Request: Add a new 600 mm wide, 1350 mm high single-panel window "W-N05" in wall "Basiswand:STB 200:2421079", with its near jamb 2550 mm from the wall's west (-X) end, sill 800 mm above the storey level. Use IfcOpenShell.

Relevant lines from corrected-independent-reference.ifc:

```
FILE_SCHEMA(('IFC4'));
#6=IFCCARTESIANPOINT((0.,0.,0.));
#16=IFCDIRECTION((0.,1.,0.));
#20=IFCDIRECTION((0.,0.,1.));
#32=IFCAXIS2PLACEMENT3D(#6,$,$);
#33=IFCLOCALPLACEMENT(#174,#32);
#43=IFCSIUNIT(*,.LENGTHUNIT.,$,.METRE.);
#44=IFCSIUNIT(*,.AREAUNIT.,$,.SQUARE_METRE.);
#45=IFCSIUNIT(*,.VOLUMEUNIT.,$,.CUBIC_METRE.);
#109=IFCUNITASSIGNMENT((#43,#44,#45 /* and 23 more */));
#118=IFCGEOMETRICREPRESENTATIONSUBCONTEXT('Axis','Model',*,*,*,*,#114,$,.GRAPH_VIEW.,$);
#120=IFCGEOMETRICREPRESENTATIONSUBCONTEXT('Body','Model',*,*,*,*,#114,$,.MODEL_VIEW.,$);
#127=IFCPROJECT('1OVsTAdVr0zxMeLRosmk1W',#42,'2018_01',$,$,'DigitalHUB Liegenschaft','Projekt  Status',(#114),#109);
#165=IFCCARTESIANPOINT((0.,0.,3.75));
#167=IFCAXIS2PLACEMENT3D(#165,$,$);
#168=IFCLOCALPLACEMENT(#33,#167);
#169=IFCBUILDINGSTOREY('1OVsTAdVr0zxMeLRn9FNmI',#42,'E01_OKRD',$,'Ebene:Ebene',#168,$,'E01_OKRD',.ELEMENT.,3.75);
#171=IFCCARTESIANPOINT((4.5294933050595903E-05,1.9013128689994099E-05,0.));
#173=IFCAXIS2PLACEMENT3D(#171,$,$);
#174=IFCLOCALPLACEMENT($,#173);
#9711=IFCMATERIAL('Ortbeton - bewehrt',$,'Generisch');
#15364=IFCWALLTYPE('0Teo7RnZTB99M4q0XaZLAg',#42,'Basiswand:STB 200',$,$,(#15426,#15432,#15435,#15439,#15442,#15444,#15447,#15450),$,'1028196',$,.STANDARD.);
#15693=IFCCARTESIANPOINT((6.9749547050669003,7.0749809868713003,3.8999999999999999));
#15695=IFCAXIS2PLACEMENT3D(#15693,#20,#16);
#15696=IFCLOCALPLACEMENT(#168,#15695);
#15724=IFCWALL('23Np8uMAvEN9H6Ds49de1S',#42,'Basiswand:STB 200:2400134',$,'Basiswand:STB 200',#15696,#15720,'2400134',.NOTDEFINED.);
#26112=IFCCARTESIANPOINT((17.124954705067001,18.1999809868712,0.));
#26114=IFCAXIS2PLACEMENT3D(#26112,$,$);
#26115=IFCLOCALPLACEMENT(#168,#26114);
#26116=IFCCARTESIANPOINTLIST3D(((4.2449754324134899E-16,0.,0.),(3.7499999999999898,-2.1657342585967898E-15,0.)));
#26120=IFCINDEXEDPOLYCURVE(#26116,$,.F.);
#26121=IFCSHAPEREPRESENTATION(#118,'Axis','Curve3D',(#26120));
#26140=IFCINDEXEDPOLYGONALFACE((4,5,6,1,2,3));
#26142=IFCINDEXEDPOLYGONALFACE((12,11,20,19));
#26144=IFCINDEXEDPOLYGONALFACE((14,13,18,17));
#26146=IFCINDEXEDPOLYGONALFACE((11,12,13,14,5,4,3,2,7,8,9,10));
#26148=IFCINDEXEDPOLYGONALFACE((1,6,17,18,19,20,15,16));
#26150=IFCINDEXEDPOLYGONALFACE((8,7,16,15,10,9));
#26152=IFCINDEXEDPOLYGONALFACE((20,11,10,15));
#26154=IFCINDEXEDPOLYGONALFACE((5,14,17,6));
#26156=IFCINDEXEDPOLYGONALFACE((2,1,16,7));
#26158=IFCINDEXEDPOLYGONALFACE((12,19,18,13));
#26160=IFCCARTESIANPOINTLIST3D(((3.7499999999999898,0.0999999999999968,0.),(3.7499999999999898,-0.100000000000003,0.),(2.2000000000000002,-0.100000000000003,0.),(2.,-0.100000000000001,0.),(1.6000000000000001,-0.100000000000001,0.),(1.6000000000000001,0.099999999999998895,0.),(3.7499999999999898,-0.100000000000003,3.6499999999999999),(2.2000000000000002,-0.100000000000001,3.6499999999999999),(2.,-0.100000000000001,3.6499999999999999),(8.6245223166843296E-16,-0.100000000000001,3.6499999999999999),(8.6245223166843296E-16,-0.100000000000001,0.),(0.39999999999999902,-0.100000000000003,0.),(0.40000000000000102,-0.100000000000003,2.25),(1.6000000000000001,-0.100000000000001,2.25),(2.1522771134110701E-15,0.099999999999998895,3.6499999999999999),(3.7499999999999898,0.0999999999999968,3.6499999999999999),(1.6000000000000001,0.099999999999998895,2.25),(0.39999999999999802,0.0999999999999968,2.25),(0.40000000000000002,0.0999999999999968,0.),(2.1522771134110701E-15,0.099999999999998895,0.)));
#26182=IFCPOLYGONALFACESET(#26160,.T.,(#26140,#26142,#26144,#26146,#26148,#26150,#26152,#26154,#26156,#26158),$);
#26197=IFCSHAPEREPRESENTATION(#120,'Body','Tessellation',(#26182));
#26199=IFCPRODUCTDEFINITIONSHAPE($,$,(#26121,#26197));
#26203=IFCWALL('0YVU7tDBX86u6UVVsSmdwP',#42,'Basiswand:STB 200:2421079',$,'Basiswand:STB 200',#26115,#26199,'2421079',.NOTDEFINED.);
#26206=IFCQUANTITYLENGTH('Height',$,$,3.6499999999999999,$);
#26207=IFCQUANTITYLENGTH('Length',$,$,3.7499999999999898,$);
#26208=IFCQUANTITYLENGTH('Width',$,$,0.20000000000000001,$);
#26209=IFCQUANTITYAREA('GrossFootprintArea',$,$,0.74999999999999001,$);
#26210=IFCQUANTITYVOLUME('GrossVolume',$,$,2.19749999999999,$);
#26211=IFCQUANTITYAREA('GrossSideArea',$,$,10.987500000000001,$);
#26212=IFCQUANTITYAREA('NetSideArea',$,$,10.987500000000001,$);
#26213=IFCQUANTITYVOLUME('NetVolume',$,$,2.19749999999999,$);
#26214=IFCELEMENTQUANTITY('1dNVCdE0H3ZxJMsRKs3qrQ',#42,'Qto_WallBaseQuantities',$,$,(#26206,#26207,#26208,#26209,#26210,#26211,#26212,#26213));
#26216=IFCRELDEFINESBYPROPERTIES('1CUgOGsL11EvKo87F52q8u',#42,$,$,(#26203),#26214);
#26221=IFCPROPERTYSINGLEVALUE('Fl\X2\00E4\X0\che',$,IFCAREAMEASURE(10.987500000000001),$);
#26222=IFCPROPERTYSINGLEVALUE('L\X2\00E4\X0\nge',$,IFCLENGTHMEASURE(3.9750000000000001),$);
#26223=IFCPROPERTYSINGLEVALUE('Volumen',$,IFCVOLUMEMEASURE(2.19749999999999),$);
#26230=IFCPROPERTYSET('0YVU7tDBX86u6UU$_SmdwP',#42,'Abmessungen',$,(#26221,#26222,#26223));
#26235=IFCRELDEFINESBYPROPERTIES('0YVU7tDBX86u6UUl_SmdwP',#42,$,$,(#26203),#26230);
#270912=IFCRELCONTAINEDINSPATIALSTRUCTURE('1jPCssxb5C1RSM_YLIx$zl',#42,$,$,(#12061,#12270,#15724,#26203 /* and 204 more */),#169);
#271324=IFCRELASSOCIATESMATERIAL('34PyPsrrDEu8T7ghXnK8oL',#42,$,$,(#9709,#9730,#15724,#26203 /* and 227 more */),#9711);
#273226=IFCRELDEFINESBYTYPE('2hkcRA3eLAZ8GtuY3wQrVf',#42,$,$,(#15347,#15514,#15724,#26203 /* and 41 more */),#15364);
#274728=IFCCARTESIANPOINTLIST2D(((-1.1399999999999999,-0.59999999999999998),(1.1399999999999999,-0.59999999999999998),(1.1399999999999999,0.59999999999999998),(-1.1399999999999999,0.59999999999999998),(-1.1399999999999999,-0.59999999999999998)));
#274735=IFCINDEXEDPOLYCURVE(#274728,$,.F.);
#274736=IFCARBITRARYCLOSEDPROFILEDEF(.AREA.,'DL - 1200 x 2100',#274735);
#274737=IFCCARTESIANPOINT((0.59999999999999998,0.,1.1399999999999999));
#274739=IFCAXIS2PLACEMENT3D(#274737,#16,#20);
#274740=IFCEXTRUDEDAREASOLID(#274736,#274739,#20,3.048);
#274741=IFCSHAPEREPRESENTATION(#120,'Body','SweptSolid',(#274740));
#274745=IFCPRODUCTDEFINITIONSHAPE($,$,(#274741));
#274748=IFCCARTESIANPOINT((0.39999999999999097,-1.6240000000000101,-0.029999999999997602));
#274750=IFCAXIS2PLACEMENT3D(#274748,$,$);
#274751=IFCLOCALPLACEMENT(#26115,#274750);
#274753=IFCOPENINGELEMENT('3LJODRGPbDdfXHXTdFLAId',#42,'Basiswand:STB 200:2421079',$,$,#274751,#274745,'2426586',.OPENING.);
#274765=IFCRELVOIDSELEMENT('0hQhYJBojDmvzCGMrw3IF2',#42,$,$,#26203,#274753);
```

```python
import numpy as np
import ifcopenshell
import ifcopenshell.api.feature
import ifcopenshell.api.geometry
import ifcopenshell.api.pset
import ifcopenshell.api.root
import ifcopenshell.api.spatial
import ifcopenshell.geom
import ifcopenshell.util.element
import ifcopenshell.util.placement
import ifcopenshell.util.representation
import ifcopenshell.util.shape
import ifcopenshell.util.unit

model = ifcopenshell.open("corrected-independent-reference.ifc")
unit_scale = ifcopenshell.util.unit.calculate_unit_scale(model)
area_scale = ifcopenshell.util.unit.calculate_unit_scale(model, "AREAUNIT")
volume_scale = ifcopenshell.util.unit.calculate_unit_scale(model, "VOLUMEUNIT")
settings = ifcopenshell.geom.settings()


def volume(element):
    """Net volume in cubic metres, openings subtracted."""
    shape = ifcopenshell.geom.create_shape(settings, element)
    return ifcopenshell.util.shape.get_volume(shape.geometry)


wall = model.by_id(26203)
storey = ifcopenshell.util.element.get_container(wall, ifc_class="IfcBuildingStorey")
context = ifcopenshell.util.representation.get_context(model, "Model", "Body", "MODEL_VIEW")
before = volume(wall)

width, height, from_end, sill = 0.6, 1.35, 2.55, 0.8  # metres

# The wall runs along its own X axis, and the end named is its -X end.
wall_shape = ifcopenshell.geom.create_shape(settings, wall)
x, y, z = ifcopenshell.util.shape.get_vertices(wall_shape.geometry).T
start = x.min() + from_end
face, thickness = float(y.min()), float(y.max() - y.min())
wall_matrix = ifcopenshell.util.placement.get_local_placement(wall.ObjectPlacement)
level = ifcopenshell.util.placement.get_local_placement(storey.ObjectPlacement)[2, 3]


def in_wall(x, y):
    """Placement at x, y metres in the wall's axes, at sill height."""
    matrix = wall_matrix.copy()
    matrix[:, 3] = wall_matrix @ np.array([x / unit_scale, y / unit_scale, 0.0, 1.0])
    matrix[2, 3] = level + sill / unit_scale
    return matrix


# Opening: a box that overshoots both wall faces by 50 mm.
opening = ifcopenshell.api.root.create_entity(model, ifc_class="IfcOpeningElement", predefined_type="OPENING")
box = ifcopenshell.api.geometry.add_wall_representation(
    model, context=context, length=width, height=height, thickness=thickness + 0.1
)
ifcopenshell.api.geometry.assign_representation(model, product=opening, representation=box)
ifcopenshell.api.geometry.edit_object_placement(model, product=opening, matrix=in_wall(start, face - 0.05), is_si=False)
ifcopenshell.api.feature.add_feature(model, feature=opening, element=wall)

window = ifcopenshell.api.root.create_entity(model, ifc_class="IfcWindow", name="W-N05", predefined_type="WINDOW")
window.OverallWidth, window.OverallHeight = width / unit_scale, height / unit_scale
window.PartitioningType = "SINGLE_PANEL"
body = ifcopenshell.api.geometry.add_window_representation(
    model,
    context=context,
    overall_width=window.OverallWidth,
    overall_height=window.OverallHeight,
    partition_type="SINGLE_PANEL",
)
ifcopenshell.api.geometry.assign_representation(model, product=window, representation=body)
ifcopenshell.api.spatial.assign_container(model, products=[window], relating_structure=storey)
ifcopenshell.api.feature.add_filling(model, opening=opening, element=window)

# Centre the window in the wall's thickness.
ifcopenshell.api.geometry.edit_object_placement(model, product=window, matrix=in_wall(start, face), is_si=False)
window_shape = ifcopenshell.geom.create_shape(settings, window)
depth = ifcopenshell.util.shape.get_vertices(window_shape.geometry)[:, 1]
offset = face + thickness / 2 - (depth.min() + depth.max()) / 2
ifcopenshell.api.geometry.edit_object_placement(model, product=window, matrix=in_wall(start, offset), is_si=False)

after = volume(wall)

# Update the wall's stored quantities.
qto = model.by_id(ifcopenshell.util.element.get_pset(wall, "Qto_WallBaseQuantities", should_inherit=False)["id"])
ifcopenshell.api.pset.edit_qto(model, qto=qto, properties={
    "NetSideArea": after / thickness / area_scale,
    "NetVolume": after / volume_scale,
})
pset = model.by_id(ifcopenshell.util.element.get_pset(wall, "Abmessungen", should_inherit=False)["id"])
ifcopenshell.api.pset.edit_pset(model, pset=pset, properties={
    "Fläche": model.create_entity("IfcAreaMeasure", after / thickness / area_scale),
    "Volumen": model.create_entity("IfcVolumeMeasure", after / volume_scale),
})

print(f"wall volume {before:.3f} -> {after:.3f} m3")

model.write("corrected-independent-reference_edited.ifc")
```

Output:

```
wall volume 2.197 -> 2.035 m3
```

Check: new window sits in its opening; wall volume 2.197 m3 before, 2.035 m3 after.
